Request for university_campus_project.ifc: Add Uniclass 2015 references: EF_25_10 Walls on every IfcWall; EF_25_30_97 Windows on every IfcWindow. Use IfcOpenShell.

First a look at what the model holds.

```python
import ifcopenshell

model = ifcopenshell.open("university_campus_project.ifc")
print(model.schema)
print("classifications:", [c.Name for c in model.by_type("IfcClassification")])
for ifc_class in ("IfcDoor", "IfcRoof", "IfcStair", "IfcWall", "IfcWindow"):
    print(ifc_class, len(model.by_type(ifc_class)))
```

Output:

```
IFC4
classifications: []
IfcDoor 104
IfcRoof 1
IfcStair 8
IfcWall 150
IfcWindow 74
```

```python
import ifcopenshell
import ifcopenshell.api.classification

model = ifcopenshell.open("university_campus_project.ifc")

system = ifcopenshell.api.classification.add_classification(model, classification="Uniclass 2015")

codes = {
    "IfcWall": ("EF_25_10", "Walls"),
    "IfcWindow": ("EF_25_30_97", "Windows"),
}
for ifc_class, (code, name) in codes.items():
    products = model.by_type(ifc_class)
    ifcopenshell.api.classification.add_reference(
        model, products=products, classification=system, identification=code, name=name
    )
    print(code, len(products))

model.write("university_campus_project_edited.ifc")
```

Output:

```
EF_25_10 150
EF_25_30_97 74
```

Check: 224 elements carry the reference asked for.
